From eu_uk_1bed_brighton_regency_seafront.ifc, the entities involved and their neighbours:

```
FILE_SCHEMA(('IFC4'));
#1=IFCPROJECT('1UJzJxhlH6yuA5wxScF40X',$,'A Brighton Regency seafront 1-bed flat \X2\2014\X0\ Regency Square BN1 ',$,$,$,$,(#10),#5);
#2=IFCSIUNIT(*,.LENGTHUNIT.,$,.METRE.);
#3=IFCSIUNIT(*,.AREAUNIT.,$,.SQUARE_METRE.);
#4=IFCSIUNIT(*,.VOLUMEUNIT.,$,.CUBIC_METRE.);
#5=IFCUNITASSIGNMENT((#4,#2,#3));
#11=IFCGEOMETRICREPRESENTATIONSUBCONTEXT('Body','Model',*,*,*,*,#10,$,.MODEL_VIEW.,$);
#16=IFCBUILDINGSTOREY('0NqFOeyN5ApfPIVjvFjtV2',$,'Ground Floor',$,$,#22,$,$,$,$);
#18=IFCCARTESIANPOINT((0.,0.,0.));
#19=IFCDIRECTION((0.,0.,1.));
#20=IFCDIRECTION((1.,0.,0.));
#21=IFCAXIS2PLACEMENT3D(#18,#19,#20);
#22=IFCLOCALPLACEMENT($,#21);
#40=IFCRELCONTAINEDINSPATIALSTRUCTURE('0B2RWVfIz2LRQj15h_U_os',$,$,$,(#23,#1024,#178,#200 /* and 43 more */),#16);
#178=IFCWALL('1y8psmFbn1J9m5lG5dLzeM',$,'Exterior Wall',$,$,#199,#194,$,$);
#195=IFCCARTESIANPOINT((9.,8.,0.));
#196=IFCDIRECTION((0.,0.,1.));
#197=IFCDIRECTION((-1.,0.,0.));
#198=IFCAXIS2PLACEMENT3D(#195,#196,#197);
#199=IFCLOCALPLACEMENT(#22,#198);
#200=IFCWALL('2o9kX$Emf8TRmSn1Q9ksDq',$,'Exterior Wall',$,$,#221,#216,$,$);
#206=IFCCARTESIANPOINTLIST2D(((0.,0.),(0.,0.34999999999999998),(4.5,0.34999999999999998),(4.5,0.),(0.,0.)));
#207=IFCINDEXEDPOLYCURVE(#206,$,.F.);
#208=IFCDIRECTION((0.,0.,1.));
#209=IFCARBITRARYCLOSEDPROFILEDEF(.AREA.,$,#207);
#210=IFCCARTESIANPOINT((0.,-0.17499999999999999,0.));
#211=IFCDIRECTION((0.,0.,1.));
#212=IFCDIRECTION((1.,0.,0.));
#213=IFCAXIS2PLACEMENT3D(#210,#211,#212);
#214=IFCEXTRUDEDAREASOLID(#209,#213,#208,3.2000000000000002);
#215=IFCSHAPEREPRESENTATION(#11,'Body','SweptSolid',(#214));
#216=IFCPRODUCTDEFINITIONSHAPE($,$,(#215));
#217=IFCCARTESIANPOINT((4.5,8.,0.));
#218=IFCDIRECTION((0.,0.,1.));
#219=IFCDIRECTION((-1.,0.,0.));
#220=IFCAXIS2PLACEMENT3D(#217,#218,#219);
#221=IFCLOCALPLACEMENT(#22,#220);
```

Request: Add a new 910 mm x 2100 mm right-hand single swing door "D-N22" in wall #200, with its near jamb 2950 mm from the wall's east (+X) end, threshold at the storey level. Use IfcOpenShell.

```python
import numpy as np
import ifcopenshell
import ifcopenshell.api.feature
import ifcopenshell.api.geometry
import ifcopenshell.api.root
import ifcopenshell.api.spatial
import ifcopenshell.geom
import ifcopenshell.util.element
import ifcopenshell.util.placement
import ifcopenshell.util.representation
import ifcopenshell.util.shape
import ifcopenshell.util.unit

model = ifcopenshell.open("eu_uk_1bed_brighton_regency_seafront.ifc")
unit_scale = ifcopenshell.util.unit.calculate_unit_scale(model)
settings = ifcopenshell.geom.settings()


def volume(element):
    """Net volume in cubic metres, openings subtracted."""
    shape = ifcopenshell.geom.create_shape(settings, element)
    return ifcopenshell.util.shape.get_volume(shape.geometry)


wall = model.by_guid("2o9kX$Emf8TRmSn1Q9ksDq")
storey = ifcopenshell.util.element.get_container(wall, ifc_class="IfcBuildingStorey")
context = ifcopenshell.util.representation.get_context(model, "Model", "Body", "MODEL_VIEW")
before = volume(wall)

width, height, from_end, sill = 0.91, 2.1, 2.95, 0.0  # metres

# The wall runs along its own X axis, and the end named is its -X end.
wall_shape = ifcopenshell.geom.create_shape(settings, wall)
x, y, z = ifcopenshell.util.shape.get_vertices(wall_shape.geometry).T
start = x.min() + from_end
face, thickness = float(y.min()), float(y.max() - y.min())
wall_matrix = ifcopenshell.util.placement.get_local_placement(wall.ObjectPlacement)
level = ifcopenshell.util.placement.get_local_placement(storey.ObjectPlacement)[2, 3]


def in_wall(x, y):
    """Placement at x, y metres in the wall's axes, at sill height."""
    matrix = wall_matrix.copy()
    matrix[:, 3] = wall_matrix @ np.array([x / unit_scale, y / unit_scale, 0.0, 1.0])
    matrix[2, 3] = level + sill / unit_scale
    return matrix


# Opening: a box that overshoots both wall faces by 50 mm.
opening = ifcopenshell.api.root.create_entity(model, ifc_class="IfcOpeningElement", predefined_type="OPENING")
box = ifcopenshell.api.geometry.add_wall_representation(
    model, context=context, length=width, height=height, thickness=thickness + 0.1
)
ifcopenshell.api.geometry.assign_representation(model, product=opening, representation=box)
ifcopenshell.api.geometry.edit_object_placement(model, product=opening, matrix=in_wall(start, face - 0.05), is_si=False)
ifcopenshell.api.feature.add_feature(model, feature=opening, element=wall)

door = ifcopenshell.api.root.create_entity(model, ifc_class="IfcDoor", name="D-N22", predefined_type="DOOR")
door.OverallWidth, door.OverallHeight = width / unit_scale, height / unit_scale
door.OperationType = "SINGLE_SWING_RIGHT"
body = ifcopenshell.api.geometry.add_door_representation(
    model,
    context=context,
    overall_width=door.OverallWidth,
    overall_height=door.OverallHeight,
    operation_type="SINGLE_SWING_RIGHT",
    lining_properties={"LiningDepth": thickness / unit_scale, "ThresholdDepth": thickness / unit_scale},
)
ifcopenshell.api.geometry.assign_representation(model, product=door, representation=body)
ifcopenshell.api.spatial.assign_container(model, products=[door], relating_structure=storey)
ifcopenshell.api.feature.add_filling(model, opening=opening, element=door)

# The lining spans the wall, so the door starts at the wall face.
ifcopenshell.api.geometry.edit_object_placement(model, product=door, matrix=in_wall(start, face), is_si=False)

after = volume(wall)

print(f"wall volume {before:.3f} -> {after:.3f} m3")

model.write("eu_uk_1bed_brighton_regency_seafront_rev.ifc")
```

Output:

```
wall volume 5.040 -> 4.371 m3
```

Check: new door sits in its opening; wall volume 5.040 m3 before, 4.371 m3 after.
